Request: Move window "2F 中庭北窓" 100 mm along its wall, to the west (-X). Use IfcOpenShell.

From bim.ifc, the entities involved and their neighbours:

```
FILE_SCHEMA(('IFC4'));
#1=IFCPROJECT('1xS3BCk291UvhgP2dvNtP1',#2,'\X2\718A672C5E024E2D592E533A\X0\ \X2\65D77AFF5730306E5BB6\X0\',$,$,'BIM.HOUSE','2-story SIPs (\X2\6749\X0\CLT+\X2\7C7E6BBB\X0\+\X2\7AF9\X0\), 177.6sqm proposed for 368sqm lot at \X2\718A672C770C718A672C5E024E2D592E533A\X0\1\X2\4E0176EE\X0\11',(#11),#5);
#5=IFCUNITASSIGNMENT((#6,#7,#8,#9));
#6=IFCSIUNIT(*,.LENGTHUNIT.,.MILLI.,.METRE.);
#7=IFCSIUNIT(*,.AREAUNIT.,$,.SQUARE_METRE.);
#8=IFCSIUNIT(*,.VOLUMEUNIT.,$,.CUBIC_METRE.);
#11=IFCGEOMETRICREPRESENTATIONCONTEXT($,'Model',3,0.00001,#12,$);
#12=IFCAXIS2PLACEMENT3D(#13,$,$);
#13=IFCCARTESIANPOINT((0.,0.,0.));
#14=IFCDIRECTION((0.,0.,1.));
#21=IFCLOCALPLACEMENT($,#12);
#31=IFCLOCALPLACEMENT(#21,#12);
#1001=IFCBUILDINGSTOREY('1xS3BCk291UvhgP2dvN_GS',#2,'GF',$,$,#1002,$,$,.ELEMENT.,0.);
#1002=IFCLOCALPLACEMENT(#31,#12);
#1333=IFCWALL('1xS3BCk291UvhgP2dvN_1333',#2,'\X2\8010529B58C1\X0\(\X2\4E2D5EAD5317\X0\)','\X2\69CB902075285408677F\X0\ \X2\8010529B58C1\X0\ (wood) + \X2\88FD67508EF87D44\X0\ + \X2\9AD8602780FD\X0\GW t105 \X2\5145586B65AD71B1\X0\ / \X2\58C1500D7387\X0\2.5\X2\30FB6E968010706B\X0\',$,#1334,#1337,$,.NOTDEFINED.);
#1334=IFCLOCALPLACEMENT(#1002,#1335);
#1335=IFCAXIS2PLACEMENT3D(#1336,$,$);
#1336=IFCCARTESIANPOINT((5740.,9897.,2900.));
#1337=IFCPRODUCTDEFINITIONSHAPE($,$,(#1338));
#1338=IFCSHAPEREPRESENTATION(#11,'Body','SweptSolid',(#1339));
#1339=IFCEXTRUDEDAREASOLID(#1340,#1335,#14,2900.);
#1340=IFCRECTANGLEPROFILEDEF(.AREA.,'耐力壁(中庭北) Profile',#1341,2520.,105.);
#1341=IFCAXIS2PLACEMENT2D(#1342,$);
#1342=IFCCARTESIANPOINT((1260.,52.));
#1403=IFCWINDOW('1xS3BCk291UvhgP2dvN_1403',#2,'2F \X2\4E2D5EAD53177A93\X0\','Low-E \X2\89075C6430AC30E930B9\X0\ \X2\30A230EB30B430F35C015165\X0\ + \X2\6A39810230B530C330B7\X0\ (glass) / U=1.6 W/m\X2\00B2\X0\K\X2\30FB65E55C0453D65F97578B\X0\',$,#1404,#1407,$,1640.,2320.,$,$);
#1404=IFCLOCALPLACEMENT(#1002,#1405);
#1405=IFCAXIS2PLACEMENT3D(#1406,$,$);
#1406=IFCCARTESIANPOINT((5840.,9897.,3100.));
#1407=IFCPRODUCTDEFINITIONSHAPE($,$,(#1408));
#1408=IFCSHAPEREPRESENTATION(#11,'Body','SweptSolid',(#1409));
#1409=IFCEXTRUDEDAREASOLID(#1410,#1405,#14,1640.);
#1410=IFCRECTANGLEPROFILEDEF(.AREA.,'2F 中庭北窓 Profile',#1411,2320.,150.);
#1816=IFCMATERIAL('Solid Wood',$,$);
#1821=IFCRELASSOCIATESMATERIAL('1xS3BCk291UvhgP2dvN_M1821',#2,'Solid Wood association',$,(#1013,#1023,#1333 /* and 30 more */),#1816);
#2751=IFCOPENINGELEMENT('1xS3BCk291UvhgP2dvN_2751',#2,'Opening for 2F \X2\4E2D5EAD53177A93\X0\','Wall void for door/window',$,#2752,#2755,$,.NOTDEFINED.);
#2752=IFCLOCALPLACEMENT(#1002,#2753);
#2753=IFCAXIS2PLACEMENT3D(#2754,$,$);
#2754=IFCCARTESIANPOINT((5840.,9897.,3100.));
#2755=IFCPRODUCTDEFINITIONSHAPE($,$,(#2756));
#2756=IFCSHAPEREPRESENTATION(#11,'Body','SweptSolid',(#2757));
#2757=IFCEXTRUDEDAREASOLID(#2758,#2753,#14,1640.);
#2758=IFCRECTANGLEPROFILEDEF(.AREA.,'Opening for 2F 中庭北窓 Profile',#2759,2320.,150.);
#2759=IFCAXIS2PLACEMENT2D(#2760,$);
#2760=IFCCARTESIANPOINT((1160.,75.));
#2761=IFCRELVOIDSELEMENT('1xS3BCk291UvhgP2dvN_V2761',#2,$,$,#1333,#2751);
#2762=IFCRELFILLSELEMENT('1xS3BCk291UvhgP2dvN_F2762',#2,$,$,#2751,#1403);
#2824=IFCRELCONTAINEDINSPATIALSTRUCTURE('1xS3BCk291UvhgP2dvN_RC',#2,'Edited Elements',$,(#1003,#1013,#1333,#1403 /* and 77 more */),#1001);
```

```python
import ifcopenshell
import ifcopenshell.api.geometry
import ifcopenshell.util.placement
import ifcopenshell.util.unit

model = ifcopenshell.open("bim.ifc")
unit_scale = ifcopenshell.util.unit.calculate_unit_scale(model)

window = model.by_id(1403)
opening = window.FillsVoids[0].RelatingOpeningElement
wall = opening.VoidsElements[0].RelatingBuildingElement

wall_matrix = ifcopenshell.util.placement.get_local_placement(wall.ObjectPlacement)
shift = wall_matrix[:3, 0] * -0.1 / unit_scale
before = ifcopenshell.util.placement.get_local_placement(window.ObjectPlacement)[:3, 3].copy()

# The window is not placed relative to its opening, so move both.
for product in (opening, window):
    matrix = ifcopenshell.util.placement.get_local_placement(product.ObjectPlacement)
    matrix[:3, 3] += shift
    ifcopenshell.api.geometry.edit_object_placement(model, product=product, matrix=matrix, is_si=False)

after = ifcopenshell.util.placement.get_local_placement(window.ObjectPlacement)[:3, 3]
print("window moved by", (after - before).round(3) + 0.0)

model.write("bim-out.ifc")
```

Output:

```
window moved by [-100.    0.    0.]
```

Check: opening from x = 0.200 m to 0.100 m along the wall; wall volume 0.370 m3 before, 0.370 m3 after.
